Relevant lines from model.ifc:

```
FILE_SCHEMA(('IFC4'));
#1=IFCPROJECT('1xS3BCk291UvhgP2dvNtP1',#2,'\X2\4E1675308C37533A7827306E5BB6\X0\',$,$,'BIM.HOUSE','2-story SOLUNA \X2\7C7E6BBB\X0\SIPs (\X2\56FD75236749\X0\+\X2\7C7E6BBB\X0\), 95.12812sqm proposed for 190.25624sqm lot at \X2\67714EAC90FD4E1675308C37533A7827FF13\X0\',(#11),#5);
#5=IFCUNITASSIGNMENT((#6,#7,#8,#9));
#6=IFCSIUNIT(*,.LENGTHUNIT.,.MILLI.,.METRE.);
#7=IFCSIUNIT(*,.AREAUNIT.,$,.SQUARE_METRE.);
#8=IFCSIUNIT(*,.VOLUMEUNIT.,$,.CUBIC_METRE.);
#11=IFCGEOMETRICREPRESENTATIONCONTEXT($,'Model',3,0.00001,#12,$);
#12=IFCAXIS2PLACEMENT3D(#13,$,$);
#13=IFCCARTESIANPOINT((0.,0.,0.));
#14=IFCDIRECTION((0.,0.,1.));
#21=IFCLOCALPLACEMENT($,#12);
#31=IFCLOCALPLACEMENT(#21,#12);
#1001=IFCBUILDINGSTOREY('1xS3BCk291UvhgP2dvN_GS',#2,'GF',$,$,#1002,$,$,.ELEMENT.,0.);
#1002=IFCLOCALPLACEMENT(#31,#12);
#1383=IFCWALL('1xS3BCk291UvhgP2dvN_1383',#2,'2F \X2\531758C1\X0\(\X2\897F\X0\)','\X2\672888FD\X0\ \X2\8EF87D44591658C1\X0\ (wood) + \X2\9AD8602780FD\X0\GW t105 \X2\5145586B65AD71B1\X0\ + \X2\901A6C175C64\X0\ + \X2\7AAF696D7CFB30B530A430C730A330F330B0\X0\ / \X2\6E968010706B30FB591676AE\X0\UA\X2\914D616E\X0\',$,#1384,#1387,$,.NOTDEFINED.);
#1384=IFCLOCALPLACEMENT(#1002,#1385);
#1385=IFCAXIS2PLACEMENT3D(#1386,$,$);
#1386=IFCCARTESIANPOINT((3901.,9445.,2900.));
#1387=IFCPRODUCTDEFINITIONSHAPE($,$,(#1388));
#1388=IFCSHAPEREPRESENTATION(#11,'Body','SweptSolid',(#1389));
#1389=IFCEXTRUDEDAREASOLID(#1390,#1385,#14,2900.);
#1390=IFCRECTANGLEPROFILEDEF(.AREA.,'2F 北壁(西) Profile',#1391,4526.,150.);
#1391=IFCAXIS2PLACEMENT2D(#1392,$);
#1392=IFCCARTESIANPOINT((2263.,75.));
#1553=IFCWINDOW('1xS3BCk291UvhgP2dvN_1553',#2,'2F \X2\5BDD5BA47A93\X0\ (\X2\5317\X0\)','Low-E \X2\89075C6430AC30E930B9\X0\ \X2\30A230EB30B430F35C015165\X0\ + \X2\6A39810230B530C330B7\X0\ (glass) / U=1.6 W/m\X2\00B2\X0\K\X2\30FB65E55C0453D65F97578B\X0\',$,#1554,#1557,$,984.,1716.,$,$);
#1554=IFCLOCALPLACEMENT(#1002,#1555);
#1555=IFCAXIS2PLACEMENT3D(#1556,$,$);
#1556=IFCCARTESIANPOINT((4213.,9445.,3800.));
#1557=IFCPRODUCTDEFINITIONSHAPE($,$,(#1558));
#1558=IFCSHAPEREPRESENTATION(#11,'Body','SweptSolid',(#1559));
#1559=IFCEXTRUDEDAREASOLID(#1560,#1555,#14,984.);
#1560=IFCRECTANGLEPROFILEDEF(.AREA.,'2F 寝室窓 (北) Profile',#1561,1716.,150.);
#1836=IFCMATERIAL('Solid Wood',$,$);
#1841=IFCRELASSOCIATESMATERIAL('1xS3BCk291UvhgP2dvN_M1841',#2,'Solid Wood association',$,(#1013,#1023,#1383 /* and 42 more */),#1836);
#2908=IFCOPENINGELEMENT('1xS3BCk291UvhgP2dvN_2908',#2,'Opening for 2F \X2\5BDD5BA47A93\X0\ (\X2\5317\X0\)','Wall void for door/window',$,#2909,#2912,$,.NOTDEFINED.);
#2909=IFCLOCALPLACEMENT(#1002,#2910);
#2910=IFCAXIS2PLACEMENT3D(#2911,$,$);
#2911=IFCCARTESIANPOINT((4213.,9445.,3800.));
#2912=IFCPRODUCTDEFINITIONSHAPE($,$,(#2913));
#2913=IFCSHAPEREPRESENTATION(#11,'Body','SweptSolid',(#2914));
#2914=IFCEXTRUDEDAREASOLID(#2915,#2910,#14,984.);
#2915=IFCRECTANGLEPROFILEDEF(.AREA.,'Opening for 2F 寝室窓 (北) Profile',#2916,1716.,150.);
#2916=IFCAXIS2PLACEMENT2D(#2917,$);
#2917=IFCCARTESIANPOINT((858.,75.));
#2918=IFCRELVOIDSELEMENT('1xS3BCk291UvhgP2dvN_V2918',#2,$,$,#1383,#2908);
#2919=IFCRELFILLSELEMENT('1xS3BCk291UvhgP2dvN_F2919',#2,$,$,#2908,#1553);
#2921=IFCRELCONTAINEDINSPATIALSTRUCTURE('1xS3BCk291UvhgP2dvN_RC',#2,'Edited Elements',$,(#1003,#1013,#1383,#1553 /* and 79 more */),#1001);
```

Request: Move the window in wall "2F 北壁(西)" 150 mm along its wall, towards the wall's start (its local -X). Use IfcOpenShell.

```python
import ifcopenshell
import ifcopenshell.api.geometry
import ifcopenshell.util.placement
import ifcopenshell.util.unit

model = ifcopenshell.open("model.ifc")
unit_scale = ifcopenshell.util.unit.calculate_unit_scale(model)

window = model.by_id(1553)
opening = window.FillsVoids[0].RelatingOpeningElement
wall = opening.VoidsElements[0].RelatingBuildingElement

wall_matrix = ifcopenshell.util.placement.get_local_placement(wall.ObjectPlacement)
shift = wall_matrix[:3, 0] * -0.15 / unit_scale
before = ifcopenshell.util.placement.get_local_placement(window.ObjectPlacement)[:3, 3].copy()

# The window is not placed relative to its opening, so move both.
for product in (opening, window):
    matrix = ifcopenshell.util.placement.get_local_placement(product.ObjectPlacement)
    matrix[:3, 3] += shift
    ifcopenshell.api.geometry.edit_object_placement(model, product=product, matrix=matrix, is_si=False)

after = ifcopenshell.util.placement.get_local_placement(window.ObjectPlacement)[:3, 3]
print("window moved by", (after - before).round(3) + 0.0)

model.write("model_rev.ifc")
```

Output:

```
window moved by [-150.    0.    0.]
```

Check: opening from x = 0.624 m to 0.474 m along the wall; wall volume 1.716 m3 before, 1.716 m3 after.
